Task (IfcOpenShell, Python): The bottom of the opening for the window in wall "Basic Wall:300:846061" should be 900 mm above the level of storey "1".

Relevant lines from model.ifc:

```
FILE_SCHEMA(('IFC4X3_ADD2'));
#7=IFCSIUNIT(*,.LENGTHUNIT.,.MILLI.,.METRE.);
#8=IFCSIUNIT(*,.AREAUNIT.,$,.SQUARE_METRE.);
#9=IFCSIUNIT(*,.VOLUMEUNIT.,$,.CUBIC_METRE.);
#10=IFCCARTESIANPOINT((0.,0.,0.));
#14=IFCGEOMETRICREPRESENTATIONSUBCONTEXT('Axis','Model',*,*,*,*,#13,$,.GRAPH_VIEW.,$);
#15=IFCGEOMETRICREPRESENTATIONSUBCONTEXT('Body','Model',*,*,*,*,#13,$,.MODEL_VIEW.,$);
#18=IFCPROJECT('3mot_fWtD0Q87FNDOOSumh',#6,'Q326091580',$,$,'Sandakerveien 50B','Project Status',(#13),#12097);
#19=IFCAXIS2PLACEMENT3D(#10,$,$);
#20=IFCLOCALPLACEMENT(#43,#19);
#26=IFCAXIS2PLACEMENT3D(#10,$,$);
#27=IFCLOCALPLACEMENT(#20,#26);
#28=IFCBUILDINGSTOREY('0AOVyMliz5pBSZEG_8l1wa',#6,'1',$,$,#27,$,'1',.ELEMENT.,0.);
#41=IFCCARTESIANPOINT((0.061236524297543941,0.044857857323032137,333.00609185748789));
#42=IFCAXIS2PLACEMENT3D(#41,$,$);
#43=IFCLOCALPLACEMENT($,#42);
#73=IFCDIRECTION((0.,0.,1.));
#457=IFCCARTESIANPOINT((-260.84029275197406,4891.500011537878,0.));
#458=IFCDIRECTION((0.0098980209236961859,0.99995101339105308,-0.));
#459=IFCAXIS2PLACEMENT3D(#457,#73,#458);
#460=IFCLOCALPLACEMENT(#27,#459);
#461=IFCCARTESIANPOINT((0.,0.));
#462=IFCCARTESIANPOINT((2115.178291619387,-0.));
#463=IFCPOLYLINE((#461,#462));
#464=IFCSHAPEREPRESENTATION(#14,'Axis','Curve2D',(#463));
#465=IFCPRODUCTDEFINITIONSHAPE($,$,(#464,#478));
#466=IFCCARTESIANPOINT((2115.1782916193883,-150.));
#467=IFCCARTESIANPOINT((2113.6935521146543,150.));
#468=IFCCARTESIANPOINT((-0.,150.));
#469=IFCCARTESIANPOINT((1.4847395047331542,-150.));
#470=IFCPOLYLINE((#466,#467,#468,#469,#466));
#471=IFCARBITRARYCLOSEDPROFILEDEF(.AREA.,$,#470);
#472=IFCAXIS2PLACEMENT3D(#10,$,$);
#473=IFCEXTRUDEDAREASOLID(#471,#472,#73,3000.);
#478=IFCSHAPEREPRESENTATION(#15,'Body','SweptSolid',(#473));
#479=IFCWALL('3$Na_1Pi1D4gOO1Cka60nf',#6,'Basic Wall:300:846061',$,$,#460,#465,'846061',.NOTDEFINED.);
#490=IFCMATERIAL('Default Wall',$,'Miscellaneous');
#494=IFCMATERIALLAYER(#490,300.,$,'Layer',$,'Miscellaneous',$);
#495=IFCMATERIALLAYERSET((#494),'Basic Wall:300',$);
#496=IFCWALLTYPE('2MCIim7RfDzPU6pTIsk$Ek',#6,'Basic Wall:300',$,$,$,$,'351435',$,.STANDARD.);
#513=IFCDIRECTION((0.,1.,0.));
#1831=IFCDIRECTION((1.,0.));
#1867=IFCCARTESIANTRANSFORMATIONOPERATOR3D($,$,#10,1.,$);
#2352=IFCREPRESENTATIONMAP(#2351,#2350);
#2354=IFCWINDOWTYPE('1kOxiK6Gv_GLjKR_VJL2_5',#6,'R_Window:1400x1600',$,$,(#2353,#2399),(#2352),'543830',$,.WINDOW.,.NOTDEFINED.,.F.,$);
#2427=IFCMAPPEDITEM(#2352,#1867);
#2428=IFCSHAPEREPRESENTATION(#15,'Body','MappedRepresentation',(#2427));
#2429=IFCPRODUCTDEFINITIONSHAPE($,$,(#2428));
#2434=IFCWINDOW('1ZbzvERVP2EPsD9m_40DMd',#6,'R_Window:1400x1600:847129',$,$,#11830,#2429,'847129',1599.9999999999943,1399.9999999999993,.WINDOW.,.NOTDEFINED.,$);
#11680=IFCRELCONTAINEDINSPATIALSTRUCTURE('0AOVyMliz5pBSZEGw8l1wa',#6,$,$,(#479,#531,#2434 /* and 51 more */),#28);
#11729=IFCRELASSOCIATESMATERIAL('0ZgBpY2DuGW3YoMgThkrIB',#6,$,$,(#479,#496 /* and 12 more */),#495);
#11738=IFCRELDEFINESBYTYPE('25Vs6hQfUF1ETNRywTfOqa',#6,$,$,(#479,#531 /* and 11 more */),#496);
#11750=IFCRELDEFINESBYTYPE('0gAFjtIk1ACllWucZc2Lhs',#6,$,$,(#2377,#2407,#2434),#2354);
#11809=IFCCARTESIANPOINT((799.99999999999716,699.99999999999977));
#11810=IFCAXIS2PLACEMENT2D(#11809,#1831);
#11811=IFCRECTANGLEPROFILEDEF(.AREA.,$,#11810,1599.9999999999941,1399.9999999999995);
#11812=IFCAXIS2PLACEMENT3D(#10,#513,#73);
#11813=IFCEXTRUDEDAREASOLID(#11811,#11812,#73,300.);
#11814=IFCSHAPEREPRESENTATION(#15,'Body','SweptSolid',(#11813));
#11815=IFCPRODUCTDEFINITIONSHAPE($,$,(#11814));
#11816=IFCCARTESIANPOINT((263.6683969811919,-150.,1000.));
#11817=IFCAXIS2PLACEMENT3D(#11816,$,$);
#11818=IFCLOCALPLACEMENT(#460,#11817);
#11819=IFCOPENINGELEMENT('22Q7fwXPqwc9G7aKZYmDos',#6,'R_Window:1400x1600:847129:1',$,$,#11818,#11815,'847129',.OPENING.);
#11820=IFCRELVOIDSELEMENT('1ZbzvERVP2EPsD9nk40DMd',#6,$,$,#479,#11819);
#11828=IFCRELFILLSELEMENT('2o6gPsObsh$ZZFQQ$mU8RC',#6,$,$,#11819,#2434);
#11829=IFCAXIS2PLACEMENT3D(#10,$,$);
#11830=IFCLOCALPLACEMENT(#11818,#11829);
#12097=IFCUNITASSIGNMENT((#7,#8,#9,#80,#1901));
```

```python
import numpy as np
import ifcopenshell
import ifcopenshell.api.geometry
import ifcopenshell.geom
import ifcopenshell.util.element
import ifcopenshell.util.placement
import ifcopenshell.util.shape
import ifcopenshell.util.unit

model = ifcopenshell.open("model.ifc")
unit_scale = ifcopenshell.util.unit.calculate_unit_scale(model)

window = model.by_guid("1ZbzvERVP2EPsD9m_40DMd")
opening = window.FillsVoids[0].RelatingOpeningElement
storey = ifcopenshell.util.element.get_container(window, ifc_class="IfcBuildingStorey")
level = ifcopenshell.util.placement.get_local_placement(storey.ObjectPlacement)[2, 3]

# The opening's origin need not be at the sill, so measure its lowest point.
shape = ifcopenshell.geom.create_shape(ifcopenshell.geom.settings(), opening)
bottom = ifcopenshell.util.shape.get_shape_bottom_elevation(shape, shape.geometry) / unit_scale
dz = level + 900.0 - bottom

shift = np.array([0.0, 0.0, dz])
# The window is placed relative to its opening, so it follows when the opening moves.
matrix = ifcopenshell.util.placement.get_local_placement(opening.ObjectPlacement)
matrix[:3, 3] += shift
ifcopenshell.api.geometry.edit_object_placement(
    model, product=opening, matrix=matrix, is_si=False, should_transform_children=True
)

print(f"moved by {dz * unit_scale:+.3f} m")

model.write("model_rev.ifc")
```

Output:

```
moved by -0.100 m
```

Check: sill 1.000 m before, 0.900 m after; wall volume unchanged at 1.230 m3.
